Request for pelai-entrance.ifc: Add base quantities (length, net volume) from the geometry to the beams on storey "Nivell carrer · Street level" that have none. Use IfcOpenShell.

First a look at what the model holds.

```python
import ifcopenshell
import ifcopenshell.util.element
import ifcopenshell.util.unit

model = ifcopenshell.open("pelai-entrance.ifc")
print(model.schema)
for unit_type in ("LENGTHUNIT", "AREAUNIT", "VOLUMEUNIT"):
    print(unit_type, ifcopenshell.util.unit.calculate_unit_scale(model, unit_type))
storey = next(s for s in model.by_type("IfcBuildingStorey") if s.Name == "Nivell carrer · Street level")
beams = [e for e in ifcopenshell.util.element.get_decomposition(storey) if e.is_a("IfcBeam")]
for e in sorted(beams, key=lambda e: e.id()):
    print(e.id(), e.is_a(), e.Name, list(ifcopenshell.util.element.get_psets(e, qtos_only=True)), sep=" | ")
```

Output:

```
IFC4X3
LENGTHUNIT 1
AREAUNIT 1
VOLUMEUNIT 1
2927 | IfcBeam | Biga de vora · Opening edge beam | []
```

```python
import ifcopenshell
import ifcopenshell.api.pset
import ifcopenshell.geom
import ifcopenshell.util.element
import ifcopenshell.util.shape
import ifcopenshell.util.unit

model = ifcopenshell.open("pelai-entrance.ifc")
unit_scale = ifcopenshell.util.unit.calculate_unit_scale(model)
volume_scale = ifcopenshell.util.unit.calculate_unit_scale(model, "VOLUMEUNIT")
settings = ifcopenshell.geom.settings()

storey = next(s for s in model.by_type("IfcBuildingStorey") if s.Name == "Nivell carrer · Street level")
beams = [e for e in ifcopenshell.util.element.get_decomposition(storey) if e.is_a("IfcBeam")]

for e in sorted(beams, key=lambda e: e.id()):
    if ifcopenshell.util.element.get_psets(e, qtos_only=True, should_inherit=False):
        continue
    # Geometry comes back in metres, in the element's own axes.
    shape = ifcopenshell.geom.create_shape(settings, e)
    values = {
        "Length": ifcopenshell.util.shape.get_max_xyz(shape.geometry) / unit_scale,
        "NetVolume": ifcopenshell.util.shape.get_volume(shape.geometry) / volume_scale,
    }
    qto = ifcopenshell.api.pset.add_qto(model, product=e, name="Qto_BeamBaseQuantities")
    ifcopenshell.api.pset.edit_qto(model, qto=qto, properties=values)
    print(e.id(), {k: round(v, 3) for k, v in values.items()})

model.write("pelai-entrance-out.ifc")
```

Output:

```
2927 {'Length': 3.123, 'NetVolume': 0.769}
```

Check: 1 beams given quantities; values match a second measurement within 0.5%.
